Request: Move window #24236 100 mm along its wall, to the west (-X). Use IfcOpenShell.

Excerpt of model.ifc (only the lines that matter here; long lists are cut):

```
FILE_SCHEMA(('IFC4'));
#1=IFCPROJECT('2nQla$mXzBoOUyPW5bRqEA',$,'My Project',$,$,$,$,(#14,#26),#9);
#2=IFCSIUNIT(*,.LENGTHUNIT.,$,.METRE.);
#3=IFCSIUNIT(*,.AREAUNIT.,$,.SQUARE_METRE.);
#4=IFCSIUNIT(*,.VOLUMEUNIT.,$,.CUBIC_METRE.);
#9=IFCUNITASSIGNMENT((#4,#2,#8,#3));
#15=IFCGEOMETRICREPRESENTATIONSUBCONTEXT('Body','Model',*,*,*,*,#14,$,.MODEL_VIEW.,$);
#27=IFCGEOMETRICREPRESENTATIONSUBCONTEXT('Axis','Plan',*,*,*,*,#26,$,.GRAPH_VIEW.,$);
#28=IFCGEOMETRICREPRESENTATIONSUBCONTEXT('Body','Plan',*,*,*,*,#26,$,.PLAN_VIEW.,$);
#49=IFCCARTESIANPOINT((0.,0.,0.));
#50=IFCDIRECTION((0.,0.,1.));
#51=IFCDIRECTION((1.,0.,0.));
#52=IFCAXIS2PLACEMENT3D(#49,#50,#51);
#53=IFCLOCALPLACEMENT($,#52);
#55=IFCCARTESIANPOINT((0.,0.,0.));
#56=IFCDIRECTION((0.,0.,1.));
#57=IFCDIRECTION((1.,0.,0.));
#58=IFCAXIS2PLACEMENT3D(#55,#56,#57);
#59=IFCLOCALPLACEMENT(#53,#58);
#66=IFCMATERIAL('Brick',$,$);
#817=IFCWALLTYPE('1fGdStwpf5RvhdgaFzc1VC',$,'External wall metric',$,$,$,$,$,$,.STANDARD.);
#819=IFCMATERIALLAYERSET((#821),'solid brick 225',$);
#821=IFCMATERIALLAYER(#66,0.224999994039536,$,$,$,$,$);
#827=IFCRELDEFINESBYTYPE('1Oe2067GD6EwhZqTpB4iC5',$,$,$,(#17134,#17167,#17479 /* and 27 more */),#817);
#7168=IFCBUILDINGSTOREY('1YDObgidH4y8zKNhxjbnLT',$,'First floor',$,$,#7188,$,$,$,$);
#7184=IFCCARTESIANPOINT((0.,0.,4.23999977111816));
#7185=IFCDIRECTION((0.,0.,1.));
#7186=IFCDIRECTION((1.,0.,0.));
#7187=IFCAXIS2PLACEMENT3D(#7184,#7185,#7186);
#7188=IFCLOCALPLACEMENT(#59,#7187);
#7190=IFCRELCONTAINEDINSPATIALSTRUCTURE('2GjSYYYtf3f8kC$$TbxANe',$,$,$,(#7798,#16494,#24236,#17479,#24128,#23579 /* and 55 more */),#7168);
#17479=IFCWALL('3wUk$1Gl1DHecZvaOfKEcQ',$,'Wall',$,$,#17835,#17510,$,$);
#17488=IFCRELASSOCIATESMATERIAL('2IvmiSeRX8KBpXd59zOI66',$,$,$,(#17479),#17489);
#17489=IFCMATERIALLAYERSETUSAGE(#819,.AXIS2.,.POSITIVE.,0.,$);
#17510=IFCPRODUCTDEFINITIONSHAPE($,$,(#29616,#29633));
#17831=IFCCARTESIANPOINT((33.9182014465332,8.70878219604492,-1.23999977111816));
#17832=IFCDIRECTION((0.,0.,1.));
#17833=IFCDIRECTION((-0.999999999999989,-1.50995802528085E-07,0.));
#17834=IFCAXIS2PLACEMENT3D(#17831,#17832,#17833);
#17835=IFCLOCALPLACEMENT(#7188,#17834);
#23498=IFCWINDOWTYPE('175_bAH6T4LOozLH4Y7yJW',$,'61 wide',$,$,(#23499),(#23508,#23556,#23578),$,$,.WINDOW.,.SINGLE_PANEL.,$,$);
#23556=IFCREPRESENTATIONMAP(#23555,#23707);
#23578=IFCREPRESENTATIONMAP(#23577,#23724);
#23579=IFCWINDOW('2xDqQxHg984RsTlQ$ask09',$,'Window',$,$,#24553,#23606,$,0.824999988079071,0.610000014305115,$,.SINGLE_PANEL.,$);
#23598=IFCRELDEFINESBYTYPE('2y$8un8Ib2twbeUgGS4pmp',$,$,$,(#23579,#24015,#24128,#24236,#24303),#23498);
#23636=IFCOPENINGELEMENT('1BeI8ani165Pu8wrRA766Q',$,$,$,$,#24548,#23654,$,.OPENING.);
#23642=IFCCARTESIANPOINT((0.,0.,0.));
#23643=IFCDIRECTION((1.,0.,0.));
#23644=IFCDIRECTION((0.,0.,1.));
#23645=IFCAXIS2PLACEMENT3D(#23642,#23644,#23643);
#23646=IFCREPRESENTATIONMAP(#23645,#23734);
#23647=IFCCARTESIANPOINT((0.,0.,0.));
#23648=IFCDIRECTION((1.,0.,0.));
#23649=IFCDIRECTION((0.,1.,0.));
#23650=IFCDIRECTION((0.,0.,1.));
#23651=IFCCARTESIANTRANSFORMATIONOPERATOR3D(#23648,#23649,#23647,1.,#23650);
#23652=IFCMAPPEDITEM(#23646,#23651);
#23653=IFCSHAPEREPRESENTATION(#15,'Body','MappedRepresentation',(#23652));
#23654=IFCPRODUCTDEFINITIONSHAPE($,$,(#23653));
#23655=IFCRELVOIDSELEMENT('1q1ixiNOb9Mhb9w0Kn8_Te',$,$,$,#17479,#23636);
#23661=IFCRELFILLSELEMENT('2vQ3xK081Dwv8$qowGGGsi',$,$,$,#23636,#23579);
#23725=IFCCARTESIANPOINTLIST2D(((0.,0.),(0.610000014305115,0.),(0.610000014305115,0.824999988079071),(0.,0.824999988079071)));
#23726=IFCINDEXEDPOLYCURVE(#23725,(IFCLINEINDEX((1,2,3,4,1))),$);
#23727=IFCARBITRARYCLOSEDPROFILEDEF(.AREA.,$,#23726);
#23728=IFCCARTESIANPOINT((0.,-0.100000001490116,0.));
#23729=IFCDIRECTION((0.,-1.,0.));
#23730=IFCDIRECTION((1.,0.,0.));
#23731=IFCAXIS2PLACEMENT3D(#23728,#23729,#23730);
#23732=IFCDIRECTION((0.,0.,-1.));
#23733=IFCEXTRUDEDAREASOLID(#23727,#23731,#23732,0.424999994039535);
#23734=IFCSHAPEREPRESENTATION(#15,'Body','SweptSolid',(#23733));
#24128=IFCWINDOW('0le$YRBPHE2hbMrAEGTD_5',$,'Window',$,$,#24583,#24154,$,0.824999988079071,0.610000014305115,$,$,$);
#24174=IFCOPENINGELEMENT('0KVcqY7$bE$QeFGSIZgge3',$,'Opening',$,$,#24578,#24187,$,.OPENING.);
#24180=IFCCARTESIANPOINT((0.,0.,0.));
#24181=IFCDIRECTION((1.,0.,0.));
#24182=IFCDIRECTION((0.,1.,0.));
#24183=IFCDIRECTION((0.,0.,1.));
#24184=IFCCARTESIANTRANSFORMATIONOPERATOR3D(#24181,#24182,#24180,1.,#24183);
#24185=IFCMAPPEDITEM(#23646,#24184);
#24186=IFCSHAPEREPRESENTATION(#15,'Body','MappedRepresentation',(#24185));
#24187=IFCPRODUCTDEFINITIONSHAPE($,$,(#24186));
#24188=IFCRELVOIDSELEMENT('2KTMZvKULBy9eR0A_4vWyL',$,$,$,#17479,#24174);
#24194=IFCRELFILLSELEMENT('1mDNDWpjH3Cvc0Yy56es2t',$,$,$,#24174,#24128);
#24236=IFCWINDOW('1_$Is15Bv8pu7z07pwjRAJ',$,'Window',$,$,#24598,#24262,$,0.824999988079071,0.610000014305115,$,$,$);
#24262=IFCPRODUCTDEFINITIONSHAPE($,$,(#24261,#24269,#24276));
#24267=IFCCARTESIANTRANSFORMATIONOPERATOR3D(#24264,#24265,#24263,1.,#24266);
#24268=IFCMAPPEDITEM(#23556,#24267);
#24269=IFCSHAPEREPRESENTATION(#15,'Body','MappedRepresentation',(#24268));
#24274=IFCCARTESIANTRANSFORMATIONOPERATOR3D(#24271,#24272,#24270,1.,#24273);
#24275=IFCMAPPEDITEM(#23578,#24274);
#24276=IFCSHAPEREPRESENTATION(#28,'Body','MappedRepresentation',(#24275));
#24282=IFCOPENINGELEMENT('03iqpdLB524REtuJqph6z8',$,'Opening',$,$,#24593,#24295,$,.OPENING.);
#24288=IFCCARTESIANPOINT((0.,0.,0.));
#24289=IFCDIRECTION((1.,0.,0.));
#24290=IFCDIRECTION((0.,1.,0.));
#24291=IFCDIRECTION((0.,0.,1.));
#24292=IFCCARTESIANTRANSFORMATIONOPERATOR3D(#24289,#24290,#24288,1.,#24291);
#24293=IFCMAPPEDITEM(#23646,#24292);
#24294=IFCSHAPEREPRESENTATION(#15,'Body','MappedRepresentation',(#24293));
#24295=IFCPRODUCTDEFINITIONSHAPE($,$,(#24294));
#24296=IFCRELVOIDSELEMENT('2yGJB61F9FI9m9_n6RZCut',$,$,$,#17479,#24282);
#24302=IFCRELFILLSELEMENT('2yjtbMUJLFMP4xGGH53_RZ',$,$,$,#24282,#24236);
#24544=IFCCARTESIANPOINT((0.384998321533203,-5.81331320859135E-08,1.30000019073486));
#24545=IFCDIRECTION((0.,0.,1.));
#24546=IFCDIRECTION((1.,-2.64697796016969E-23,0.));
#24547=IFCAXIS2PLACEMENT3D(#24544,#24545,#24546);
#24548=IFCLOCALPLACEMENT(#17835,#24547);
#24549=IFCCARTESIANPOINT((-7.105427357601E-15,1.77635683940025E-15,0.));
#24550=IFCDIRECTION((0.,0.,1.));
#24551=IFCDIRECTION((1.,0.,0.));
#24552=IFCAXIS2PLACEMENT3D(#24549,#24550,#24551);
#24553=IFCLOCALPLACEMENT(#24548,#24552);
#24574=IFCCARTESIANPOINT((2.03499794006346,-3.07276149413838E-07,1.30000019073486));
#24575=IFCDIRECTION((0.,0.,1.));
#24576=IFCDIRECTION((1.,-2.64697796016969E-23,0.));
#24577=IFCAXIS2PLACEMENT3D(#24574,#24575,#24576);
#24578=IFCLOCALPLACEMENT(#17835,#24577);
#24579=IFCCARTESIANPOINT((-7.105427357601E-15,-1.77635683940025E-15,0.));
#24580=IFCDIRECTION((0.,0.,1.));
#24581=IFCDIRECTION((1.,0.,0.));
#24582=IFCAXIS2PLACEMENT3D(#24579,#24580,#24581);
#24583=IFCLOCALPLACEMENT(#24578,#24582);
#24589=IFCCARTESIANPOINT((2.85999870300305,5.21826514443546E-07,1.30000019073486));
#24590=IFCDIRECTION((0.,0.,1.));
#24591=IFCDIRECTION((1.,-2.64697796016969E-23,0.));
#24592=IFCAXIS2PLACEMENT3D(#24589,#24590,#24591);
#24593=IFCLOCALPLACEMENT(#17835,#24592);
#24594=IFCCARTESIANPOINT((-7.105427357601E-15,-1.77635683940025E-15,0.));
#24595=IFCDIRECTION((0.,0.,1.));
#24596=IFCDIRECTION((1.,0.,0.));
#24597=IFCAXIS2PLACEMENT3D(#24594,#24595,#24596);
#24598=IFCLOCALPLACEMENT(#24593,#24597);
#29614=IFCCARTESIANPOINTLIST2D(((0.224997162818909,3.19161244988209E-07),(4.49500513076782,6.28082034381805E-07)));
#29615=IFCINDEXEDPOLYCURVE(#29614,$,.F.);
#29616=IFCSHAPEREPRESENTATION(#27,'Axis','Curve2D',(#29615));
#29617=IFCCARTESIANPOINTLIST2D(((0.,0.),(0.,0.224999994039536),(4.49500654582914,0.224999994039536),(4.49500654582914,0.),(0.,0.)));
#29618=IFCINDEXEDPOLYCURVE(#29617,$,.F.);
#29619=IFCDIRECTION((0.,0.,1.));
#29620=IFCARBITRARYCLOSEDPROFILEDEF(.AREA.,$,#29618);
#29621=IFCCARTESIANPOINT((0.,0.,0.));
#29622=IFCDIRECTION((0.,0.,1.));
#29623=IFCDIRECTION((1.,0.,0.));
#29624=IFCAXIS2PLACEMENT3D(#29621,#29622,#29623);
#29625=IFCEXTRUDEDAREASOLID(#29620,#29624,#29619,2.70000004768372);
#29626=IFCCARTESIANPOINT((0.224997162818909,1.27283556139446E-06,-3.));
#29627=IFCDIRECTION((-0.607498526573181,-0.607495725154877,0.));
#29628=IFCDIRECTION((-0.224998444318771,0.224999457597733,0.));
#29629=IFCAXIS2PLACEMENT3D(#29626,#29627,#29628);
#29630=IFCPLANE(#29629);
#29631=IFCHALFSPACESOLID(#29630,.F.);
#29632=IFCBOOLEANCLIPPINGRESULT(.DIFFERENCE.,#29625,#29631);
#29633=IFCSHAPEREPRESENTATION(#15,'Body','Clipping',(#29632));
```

```python
import ifcopenshell
import ifcopenshell.api.geometry
import ifcopenshell.util.placement
import ifcopenshell.util.unit

model = ifcopenshell.open("model.ifc")
unit_scale = ifcopenshell.util.unit.calculate_unit_scale(model)

window = model.by_guid("1_$Is15Bv8pu7z07pwjRAJ")
opening = window.FillsVoids[0].RelatingOpeningElement
wall = opening.VoidsElements[0].RelatingBuildingElement

wall_matrix = ifcopenshell.util.placement.get_local_placement(wall.ObjectPlacement)
shift = wall_matrix[:3, 0] * 0.1 / unit_scale
before = ifcopenshell.util.placement.get_local_placement(window.ObjectPlacement)[:3, 3].copy()

# The window is placed relative to its opening, so it follows when the opening moves.
matrix = ifcopenshell.util.placement.get_local_placement(opening.ObjectPlacement)
matrix[:3, 3] += shift
ifcopenshell.api.geometry.edit_object_placement(
    model, product=opening, matrix=matrix, is_si=False, should_transform_children=True
)

after = ifcopenshell.util.placement.get_local_placement(window.ObjectPlacement)[:3, 3]
print("window moved by", (after - before).round(3) + 0.0)

model.write("model_updated.ifc")
```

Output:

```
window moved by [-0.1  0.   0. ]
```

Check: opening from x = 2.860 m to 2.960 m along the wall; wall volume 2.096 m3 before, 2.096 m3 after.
